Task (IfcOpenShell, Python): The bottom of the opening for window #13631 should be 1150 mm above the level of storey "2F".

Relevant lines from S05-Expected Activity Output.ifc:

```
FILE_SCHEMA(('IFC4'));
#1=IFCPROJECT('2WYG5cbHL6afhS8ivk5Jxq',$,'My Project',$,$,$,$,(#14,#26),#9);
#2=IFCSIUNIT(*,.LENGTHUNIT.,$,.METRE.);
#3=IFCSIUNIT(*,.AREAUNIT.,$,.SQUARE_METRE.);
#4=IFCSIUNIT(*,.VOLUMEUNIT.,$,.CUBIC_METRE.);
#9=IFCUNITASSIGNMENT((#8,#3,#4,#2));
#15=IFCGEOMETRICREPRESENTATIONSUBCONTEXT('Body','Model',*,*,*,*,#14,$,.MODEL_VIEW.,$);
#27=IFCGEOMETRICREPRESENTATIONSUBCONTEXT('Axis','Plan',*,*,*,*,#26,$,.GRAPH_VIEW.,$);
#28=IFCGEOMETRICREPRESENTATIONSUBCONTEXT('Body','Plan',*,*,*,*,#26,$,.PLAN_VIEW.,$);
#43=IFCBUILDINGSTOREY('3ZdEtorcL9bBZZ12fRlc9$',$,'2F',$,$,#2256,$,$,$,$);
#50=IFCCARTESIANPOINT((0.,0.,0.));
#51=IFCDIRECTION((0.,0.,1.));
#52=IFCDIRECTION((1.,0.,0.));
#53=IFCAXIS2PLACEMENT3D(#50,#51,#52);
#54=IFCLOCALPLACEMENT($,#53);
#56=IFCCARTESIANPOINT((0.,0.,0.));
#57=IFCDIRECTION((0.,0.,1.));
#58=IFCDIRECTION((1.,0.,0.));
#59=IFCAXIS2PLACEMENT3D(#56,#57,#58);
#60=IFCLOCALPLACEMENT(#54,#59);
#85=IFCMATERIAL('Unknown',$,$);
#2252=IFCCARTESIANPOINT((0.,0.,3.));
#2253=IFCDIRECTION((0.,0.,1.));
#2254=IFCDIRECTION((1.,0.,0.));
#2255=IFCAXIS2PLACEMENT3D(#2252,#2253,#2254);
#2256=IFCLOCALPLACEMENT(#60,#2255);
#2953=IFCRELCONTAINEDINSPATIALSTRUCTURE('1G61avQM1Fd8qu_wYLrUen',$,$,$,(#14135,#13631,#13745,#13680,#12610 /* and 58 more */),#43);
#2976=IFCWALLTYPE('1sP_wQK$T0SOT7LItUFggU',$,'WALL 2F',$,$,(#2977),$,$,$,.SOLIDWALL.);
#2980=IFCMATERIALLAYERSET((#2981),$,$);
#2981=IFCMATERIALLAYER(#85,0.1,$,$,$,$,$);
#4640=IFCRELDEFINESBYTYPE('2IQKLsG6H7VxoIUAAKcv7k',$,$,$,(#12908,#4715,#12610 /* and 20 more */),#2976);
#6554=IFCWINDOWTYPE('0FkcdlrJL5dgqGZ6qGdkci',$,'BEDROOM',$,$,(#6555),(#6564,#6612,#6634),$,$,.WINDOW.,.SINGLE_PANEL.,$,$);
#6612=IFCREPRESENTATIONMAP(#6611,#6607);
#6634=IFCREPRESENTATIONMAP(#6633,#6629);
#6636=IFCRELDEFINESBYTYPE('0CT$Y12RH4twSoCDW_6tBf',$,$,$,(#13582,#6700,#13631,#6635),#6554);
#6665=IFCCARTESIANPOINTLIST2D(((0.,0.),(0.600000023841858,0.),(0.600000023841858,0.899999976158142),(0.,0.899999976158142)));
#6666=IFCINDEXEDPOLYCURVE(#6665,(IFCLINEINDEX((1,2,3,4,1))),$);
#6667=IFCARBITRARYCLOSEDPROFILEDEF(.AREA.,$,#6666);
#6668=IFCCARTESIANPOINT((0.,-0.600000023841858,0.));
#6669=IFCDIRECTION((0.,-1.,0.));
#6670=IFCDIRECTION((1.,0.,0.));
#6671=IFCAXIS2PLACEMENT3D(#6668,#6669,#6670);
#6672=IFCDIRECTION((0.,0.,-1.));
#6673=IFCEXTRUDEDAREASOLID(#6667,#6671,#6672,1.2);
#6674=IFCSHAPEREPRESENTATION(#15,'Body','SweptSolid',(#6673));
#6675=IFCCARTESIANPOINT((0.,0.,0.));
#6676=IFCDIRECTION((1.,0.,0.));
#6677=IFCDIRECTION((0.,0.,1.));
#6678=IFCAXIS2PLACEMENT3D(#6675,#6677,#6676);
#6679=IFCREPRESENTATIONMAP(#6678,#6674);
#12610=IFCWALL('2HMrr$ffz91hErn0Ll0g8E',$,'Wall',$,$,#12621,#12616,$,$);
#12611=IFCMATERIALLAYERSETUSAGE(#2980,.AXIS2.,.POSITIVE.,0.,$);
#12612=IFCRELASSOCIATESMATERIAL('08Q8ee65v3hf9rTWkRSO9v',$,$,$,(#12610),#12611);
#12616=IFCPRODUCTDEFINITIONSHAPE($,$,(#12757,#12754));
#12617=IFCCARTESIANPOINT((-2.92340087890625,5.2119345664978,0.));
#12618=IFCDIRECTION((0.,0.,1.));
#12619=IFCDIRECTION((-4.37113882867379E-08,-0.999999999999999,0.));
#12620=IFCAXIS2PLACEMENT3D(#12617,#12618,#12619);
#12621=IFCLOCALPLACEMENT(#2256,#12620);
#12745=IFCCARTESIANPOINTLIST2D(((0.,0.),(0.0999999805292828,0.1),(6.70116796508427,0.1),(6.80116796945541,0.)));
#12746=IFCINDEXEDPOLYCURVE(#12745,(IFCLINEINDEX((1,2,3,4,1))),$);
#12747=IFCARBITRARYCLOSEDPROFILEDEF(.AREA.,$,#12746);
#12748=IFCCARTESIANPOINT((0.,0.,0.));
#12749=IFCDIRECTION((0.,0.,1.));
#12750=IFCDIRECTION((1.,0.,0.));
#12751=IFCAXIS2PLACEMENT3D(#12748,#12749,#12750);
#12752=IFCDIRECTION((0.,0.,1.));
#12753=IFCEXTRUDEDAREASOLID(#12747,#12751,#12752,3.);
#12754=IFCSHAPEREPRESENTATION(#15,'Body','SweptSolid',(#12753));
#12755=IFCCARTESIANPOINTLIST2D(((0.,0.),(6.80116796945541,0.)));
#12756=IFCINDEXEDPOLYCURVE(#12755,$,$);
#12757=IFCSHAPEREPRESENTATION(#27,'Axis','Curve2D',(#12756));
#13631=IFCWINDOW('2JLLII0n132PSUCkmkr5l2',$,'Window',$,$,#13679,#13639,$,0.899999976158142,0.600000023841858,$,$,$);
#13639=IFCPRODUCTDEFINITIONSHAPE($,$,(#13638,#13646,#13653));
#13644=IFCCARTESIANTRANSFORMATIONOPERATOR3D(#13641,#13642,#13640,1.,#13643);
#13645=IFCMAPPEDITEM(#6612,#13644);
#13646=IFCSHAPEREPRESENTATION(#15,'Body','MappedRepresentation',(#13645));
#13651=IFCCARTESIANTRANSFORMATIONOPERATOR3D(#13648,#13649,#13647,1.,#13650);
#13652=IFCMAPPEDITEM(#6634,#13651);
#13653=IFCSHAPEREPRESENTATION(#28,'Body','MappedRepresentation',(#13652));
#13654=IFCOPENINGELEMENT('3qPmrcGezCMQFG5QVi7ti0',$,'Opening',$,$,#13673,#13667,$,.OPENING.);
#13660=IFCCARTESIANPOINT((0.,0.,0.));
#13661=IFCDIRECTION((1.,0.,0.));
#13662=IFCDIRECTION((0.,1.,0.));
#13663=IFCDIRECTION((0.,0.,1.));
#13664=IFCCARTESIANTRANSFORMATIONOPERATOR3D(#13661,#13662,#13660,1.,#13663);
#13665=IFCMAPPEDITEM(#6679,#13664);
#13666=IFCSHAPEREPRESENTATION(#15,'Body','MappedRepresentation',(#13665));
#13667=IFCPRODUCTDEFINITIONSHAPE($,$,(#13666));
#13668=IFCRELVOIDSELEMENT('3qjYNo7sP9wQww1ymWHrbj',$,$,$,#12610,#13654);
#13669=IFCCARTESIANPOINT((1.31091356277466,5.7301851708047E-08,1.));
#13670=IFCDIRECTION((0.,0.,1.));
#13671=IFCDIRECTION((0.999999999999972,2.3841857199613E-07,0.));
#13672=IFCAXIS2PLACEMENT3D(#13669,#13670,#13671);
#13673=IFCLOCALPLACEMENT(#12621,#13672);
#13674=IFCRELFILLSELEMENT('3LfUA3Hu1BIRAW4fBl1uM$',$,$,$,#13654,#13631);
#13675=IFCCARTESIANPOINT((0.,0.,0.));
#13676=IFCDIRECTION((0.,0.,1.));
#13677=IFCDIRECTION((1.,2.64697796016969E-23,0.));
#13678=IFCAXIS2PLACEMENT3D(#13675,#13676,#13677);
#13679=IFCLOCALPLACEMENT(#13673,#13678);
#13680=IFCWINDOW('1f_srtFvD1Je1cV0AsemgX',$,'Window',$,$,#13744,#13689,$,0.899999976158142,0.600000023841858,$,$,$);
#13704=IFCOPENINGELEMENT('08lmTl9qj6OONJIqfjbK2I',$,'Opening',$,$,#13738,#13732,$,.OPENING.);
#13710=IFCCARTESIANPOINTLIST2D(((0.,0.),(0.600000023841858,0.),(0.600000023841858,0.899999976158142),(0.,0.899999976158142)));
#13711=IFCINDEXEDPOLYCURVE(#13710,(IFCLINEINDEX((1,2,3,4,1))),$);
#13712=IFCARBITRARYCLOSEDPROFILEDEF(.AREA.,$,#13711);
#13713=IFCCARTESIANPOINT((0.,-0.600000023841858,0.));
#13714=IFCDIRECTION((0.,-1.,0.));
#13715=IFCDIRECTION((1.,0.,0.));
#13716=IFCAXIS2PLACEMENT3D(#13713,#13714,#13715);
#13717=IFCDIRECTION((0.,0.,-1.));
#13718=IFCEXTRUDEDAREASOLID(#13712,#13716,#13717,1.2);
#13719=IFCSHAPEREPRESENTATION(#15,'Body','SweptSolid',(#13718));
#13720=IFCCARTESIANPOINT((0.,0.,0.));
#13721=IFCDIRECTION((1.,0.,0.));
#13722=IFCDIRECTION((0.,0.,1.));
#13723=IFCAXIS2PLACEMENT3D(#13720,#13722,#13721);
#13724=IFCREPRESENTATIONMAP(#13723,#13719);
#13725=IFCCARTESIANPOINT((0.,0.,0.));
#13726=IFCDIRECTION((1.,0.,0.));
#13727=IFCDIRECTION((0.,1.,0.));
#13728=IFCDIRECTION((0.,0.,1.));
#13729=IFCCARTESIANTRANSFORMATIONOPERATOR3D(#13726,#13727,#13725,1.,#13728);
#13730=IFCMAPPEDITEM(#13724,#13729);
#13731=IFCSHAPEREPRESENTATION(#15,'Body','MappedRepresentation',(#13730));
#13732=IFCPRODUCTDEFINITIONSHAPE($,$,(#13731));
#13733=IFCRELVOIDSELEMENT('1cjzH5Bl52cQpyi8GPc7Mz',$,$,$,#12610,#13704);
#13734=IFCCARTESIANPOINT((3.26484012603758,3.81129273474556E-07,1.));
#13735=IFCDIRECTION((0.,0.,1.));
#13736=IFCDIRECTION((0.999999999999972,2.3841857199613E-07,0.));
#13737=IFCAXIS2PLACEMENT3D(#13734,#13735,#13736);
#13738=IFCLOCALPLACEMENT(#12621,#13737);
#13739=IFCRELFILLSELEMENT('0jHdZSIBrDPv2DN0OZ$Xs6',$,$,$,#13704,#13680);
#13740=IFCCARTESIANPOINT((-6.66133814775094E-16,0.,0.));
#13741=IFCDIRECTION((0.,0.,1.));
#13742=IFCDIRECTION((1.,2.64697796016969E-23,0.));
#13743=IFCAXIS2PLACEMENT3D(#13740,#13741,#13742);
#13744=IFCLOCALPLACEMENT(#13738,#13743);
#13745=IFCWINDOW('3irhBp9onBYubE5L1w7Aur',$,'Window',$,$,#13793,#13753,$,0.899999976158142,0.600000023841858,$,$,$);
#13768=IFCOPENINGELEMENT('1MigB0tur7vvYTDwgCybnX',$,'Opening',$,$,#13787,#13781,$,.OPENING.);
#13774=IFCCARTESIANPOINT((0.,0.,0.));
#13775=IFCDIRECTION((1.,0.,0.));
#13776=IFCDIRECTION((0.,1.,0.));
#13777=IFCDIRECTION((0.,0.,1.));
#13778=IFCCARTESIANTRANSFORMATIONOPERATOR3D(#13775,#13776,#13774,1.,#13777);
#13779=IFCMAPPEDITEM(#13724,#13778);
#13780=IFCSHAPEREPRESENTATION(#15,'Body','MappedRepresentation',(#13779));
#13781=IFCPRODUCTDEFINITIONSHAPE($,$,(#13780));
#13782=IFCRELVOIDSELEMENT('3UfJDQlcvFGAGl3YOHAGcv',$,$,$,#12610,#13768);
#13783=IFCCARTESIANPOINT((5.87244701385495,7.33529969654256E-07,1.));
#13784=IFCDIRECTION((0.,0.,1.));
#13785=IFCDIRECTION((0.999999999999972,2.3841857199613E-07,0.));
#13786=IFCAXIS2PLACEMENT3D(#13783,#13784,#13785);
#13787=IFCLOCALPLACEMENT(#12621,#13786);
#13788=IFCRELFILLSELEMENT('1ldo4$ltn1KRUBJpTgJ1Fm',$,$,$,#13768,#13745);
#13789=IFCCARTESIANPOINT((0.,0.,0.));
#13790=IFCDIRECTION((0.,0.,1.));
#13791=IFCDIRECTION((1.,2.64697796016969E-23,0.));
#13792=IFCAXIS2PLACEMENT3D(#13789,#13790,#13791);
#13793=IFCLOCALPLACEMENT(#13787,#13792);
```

```python
import numpy as np
import ifcopenshell
import ifcopenshell.api.geometry
import ifcopenshell.geom
import ifcopenshell.util.element
import ifcopenshell.util.placement
import ifcopenshell.util.shape
import ifcopenshell.util.unit

model = ifcopenshell.open("S05-Expected Activity Output.ifc")
unit_scale = ifcopenshell.util.unit.calculate_unit_scale(model)

window = model.by_guid("2JLLII0n132PSUCkmkr5l2")
opening = window.FillsVoids[0].RelatingOpeningElement
storey = ifcopenshell.util.element.get_container(window, ifc_class="IfcBuildingStorey")
level = ifcopenshell.util.placement.get_local_placement(storey.ObjectPlacement)[2, 3]

# The opening's origin need not be at the sill, so measure its lowest point.
shape = ifcopenshell.geom.create_shape(ifcopenshell.geom.settings(), opening)
bottom = ifcopenshell.util.shape.get_shape_bottom_elevation(shape, shape.geometry) / unit_scale
dz = level + 1.15 / unit_scale - bottom

shift = np.array([0.0, 0.0, dz])
# The window is placed relative to its opening, so it follows when the opening moves.
matrix = ifcopenshell.util.placement.get_local_placement(opening.ObjectPlacement)
matrix[:3, 3] += shift
ifcopenshell.api.geometry.edit_object_placement(
    model, product=opening, matrix=matrix, is_si=False, should_transform_children=True
)

print(f"moved by {dz * unit_scale:+.3f} m")

model.write("S05-Expected Activity Output_rev.ifc")
```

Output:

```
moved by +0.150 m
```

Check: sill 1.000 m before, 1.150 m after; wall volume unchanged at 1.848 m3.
